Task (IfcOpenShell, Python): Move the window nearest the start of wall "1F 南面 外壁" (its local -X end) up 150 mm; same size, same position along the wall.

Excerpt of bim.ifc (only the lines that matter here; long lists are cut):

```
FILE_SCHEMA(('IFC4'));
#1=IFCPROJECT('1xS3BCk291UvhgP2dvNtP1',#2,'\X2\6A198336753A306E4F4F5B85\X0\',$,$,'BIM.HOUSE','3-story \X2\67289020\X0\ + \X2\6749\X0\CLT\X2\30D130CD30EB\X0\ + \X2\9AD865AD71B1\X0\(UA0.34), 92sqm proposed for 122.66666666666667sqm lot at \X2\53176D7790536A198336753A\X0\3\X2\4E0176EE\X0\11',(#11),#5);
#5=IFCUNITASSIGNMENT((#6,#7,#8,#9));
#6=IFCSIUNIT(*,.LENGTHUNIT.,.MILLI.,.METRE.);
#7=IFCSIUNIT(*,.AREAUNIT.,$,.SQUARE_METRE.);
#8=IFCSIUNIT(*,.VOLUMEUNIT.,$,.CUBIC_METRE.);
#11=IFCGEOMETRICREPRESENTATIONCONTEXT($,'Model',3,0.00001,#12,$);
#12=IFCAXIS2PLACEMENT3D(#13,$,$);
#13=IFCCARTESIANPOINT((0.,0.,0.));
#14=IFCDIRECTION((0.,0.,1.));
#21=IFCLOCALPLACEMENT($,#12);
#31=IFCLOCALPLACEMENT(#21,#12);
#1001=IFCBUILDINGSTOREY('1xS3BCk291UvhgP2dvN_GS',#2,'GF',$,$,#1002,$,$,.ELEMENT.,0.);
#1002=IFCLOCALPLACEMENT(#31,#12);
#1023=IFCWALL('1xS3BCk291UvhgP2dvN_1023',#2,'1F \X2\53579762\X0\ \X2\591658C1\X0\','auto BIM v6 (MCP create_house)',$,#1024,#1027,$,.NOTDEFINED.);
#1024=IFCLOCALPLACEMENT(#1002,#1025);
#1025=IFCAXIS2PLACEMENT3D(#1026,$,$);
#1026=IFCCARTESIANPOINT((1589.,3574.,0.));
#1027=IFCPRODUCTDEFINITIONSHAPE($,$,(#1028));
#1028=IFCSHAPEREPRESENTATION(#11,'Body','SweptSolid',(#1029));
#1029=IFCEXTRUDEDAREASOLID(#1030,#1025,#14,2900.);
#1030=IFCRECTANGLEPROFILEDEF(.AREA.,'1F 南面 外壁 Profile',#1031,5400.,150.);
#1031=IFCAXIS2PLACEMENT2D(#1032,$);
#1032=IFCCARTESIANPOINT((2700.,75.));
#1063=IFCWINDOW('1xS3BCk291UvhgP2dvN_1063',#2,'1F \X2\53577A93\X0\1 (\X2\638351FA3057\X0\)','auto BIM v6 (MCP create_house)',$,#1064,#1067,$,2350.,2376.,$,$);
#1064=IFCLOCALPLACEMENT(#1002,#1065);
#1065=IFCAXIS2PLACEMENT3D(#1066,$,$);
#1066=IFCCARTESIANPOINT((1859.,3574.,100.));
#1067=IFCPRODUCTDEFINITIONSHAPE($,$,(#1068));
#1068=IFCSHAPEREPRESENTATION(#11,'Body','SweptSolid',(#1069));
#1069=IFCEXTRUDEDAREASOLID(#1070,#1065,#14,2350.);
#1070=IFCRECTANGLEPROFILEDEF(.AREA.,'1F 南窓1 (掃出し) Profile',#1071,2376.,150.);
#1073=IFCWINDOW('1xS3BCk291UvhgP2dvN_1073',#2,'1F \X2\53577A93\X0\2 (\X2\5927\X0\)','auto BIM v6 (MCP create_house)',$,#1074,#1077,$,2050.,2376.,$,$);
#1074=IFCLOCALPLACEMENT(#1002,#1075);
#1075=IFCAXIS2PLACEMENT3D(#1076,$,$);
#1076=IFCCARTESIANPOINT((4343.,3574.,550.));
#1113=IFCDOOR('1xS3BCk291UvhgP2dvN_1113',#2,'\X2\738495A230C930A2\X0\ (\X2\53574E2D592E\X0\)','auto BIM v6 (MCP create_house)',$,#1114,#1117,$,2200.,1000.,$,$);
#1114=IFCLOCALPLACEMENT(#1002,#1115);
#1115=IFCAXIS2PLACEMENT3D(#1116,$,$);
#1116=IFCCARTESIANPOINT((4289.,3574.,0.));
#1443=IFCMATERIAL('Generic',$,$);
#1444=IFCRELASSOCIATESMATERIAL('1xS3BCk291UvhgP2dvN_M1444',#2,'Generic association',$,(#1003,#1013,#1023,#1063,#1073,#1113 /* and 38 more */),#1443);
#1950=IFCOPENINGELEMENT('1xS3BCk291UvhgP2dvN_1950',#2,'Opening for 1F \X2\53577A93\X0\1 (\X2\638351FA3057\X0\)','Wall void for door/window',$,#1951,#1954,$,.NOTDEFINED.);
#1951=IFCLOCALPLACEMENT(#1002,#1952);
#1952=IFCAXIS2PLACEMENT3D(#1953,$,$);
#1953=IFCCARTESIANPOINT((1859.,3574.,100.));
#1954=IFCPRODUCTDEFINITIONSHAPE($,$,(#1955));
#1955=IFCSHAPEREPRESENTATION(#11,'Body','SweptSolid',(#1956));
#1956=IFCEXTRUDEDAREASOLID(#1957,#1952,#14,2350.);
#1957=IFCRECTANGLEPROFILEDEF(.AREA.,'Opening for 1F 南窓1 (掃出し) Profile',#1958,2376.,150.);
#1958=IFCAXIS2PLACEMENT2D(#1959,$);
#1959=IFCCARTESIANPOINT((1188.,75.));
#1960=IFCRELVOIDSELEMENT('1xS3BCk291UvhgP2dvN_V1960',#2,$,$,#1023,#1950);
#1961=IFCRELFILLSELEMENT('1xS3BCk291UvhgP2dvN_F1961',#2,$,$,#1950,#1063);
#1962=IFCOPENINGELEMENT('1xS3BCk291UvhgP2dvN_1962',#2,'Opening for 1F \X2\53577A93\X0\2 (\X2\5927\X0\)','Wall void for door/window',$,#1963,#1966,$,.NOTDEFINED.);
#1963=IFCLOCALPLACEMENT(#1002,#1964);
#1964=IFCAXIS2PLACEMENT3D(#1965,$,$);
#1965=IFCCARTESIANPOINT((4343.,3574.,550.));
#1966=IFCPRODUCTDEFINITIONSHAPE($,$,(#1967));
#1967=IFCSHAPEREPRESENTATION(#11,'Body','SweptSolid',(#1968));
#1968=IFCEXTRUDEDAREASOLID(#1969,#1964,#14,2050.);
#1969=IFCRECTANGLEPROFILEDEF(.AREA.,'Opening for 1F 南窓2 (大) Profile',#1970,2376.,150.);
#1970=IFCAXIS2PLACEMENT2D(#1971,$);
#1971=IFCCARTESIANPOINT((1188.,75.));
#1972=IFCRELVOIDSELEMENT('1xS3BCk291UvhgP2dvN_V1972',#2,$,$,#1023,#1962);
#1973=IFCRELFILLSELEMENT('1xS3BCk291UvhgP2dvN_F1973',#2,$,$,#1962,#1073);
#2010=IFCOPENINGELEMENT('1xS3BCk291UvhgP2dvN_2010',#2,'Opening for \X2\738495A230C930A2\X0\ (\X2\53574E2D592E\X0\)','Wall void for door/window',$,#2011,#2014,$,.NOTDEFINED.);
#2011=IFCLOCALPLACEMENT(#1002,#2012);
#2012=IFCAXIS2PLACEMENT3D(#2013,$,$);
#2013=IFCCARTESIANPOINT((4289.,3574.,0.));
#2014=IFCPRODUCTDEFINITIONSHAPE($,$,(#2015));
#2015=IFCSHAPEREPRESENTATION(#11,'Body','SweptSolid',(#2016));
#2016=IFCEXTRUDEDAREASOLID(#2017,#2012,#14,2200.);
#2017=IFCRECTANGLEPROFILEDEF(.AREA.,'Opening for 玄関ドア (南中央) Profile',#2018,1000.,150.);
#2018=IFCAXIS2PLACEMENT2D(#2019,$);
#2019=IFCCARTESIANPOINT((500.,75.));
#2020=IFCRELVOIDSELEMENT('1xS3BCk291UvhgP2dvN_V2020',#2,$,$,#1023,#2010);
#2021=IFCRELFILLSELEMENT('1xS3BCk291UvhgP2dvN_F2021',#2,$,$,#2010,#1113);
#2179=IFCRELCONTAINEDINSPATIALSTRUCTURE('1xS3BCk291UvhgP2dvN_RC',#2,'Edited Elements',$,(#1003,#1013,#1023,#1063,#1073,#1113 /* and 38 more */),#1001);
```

```python
import numpy as np
import ifcopenshell
import ifcopenshell.api.geometry
import ifcopenshell.util.placement
import ifcopenshell.util.unit

model = ifcopenshell.open("bim.ifc")
unit_scale = ifcopenshell.util.unit.calculate_unit_scale(model)

window = model.by_guid("1xS3BCk291UvhgP2dvN_1063")
opening = window.FillsVoids[0].RelatingOpeningElement
dz = 0.15 / unit_scale

shift = np.array([0.0, 0.0, dz])
# The window is not placed relative to its opening, so move both.
for product in (opening, window):
    matrix = ifcopenshell.util.placement.get_local_placement(product.ObjectPlacement)
    matrix[:3, 3] += shift
    ifcopenshell.api.geometry.edit_object_placement(model, product=product, matrix=matrix, is_si=False)

print(f"moved by {dz * unit_scale:+.3f} m")

model.write("bim_updated.ifc")
```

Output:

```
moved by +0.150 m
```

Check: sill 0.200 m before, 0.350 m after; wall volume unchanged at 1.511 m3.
